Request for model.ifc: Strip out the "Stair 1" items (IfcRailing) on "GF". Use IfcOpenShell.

First a look at what the model holds.

```python
import ifcopenshell
import ifcopenshell.util.element

model = ifcopenshell.open("model.ifc")
print(model.schema)
storey = next(s for s in model.by_type("IfcBuildingStorey") if s.Name == "GF")
railings = [e for e in ifcopenshell.util.element.get_decomposition(storey) if e.is_a("IfcRailing")]
seen = {}
for e in railings:
    element_type = ifcopenshell.util.element.get_type(e)
    name = element_type.Name if element_type not in (None, e) else None
    seen[name] = seen.get(name, 0) + 1
for name, count in sorted(seen.items(), key=str):
    print(count, "x", name)
```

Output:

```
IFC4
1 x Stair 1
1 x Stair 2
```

```python
import ifcopenshell
import ifcopenshell.api.root
import ifcopenshell.util.element

model = ifcopenshell.open("model.ifc")

storey = next(s for s in model.by_type("IfcBuildingStorey") if s.Name == "GF")
railings = [e for e in ifcopenshell.util.element.get_decomposition(storey) if e.is_a("IfcRailing")]
targets = [e for e in railings if (t := ifcopenshell.util.element.get_type(e)) not in (None, e) and t.Name == "Stair 1"]

for e in targets:
    ifcopenshell.api.root.remove_product(model, product=e)
print(len(targets), "removed")

model.write("model_v2.ifc")
```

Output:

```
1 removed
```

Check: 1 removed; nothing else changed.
